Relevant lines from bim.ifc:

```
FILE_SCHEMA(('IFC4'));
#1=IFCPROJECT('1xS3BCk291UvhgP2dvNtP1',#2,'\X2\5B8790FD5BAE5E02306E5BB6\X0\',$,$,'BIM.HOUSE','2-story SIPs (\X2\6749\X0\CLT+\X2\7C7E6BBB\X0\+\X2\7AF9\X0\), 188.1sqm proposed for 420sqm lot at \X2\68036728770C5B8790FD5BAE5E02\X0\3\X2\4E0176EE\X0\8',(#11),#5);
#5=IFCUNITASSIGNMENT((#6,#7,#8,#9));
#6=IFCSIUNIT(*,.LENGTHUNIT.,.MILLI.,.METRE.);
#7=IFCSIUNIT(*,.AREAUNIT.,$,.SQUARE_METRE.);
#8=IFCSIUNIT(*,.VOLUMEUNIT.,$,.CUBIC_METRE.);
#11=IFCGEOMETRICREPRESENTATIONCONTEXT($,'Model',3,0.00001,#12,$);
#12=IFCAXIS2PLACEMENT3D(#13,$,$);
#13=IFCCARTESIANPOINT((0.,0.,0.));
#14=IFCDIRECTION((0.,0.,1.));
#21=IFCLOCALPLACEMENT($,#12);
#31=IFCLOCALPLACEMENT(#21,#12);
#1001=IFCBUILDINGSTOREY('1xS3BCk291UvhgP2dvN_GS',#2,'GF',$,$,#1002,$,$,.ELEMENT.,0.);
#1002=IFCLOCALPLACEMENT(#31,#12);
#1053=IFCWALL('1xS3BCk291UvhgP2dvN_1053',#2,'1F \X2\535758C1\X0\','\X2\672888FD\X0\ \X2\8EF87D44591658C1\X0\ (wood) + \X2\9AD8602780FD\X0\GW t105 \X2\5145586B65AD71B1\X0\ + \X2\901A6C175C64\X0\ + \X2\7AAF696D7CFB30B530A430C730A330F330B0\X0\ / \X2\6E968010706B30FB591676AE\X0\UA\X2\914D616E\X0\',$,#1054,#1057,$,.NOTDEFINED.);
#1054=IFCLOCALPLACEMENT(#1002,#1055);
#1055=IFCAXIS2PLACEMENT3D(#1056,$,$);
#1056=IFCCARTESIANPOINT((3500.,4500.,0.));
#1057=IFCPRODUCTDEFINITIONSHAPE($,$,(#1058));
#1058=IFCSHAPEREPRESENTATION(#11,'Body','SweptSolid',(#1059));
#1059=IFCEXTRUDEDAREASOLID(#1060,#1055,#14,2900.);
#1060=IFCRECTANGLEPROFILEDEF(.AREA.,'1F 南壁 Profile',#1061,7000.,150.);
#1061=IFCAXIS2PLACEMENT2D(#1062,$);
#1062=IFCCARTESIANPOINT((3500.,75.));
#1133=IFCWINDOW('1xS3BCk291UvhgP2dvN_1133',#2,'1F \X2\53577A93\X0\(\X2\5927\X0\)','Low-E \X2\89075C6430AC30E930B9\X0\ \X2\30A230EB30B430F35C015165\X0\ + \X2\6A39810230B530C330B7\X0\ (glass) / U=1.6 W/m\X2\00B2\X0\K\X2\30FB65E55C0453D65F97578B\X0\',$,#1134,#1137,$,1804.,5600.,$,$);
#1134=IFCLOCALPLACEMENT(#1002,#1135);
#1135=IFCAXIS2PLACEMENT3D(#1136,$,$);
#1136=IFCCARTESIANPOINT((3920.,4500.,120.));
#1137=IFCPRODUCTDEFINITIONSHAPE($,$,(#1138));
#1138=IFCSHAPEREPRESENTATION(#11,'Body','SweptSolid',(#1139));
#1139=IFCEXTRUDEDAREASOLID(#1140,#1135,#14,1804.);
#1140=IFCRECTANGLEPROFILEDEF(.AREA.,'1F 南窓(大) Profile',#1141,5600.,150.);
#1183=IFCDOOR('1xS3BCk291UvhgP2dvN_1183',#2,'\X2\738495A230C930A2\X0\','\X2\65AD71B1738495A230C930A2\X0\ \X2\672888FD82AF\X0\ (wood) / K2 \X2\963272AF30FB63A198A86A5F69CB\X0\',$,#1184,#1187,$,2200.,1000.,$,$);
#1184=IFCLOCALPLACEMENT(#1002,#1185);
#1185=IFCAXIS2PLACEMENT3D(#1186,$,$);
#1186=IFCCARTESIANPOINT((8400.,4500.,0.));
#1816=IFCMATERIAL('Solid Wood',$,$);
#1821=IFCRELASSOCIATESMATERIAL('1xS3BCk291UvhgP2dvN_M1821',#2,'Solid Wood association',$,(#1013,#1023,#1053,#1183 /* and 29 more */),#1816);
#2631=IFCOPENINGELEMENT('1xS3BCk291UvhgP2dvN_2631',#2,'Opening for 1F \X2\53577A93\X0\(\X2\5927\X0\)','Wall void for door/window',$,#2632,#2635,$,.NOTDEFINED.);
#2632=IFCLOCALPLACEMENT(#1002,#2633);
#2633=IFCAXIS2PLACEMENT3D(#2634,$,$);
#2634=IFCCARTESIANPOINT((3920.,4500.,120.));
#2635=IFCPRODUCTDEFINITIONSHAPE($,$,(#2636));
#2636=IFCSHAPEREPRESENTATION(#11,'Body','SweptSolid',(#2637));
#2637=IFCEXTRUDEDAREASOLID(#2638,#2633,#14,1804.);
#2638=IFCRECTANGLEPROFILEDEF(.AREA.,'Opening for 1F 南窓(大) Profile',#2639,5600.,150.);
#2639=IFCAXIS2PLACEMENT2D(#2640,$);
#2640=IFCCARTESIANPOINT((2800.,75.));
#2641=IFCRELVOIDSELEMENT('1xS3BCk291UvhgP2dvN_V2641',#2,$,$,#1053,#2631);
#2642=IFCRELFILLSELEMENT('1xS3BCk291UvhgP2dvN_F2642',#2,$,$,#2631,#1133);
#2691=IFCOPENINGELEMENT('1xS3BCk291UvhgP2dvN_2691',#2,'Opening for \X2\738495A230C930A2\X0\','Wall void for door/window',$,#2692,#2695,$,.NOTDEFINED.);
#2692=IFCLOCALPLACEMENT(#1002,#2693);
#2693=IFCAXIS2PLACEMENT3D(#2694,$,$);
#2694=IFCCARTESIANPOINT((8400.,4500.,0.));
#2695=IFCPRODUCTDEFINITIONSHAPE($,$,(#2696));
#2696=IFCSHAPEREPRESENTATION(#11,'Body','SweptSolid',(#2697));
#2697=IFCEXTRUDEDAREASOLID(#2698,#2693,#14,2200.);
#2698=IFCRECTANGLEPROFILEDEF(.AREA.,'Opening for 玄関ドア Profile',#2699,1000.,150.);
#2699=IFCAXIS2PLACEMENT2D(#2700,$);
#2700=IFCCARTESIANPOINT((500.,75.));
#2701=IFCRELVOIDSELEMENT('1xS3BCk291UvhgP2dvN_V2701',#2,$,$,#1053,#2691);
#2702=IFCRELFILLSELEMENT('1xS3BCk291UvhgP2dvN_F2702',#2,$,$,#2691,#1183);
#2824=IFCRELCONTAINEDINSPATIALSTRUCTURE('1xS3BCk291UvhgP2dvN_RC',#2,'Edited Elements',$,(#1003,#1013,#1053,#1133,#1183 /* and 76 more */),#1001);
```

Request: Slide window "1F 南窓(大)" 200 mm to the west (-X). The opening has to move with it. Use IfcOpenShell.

```python
import ifcopenshell
import ifcopenshell.api.geometry
import ifcopenshell.util.placement
import ifcopenshell.util.unit

model = ifcopenshell.open("bim.ifc")
unit_scale = ifcopenshell.util.unit.calculate_unit_scale(model)

window = model.by_guid("1xS3BCk291UvhgP2dvN_1133")
opening = window.FillsVoids[0].RelatingOpeningElement
wall = opening.VoidsElements[0].RelatingBuildingElement

wall_matrix = ifcopenshell.util.placement.get_local_placement(wall.ObjectPlacement)
shift = wall_matrix[:3, 0] * -0.2 / unit_scale
before = ifcopenshell.util.placement.get_local_placement(window.ObjectPlacement)[:3, 3].copy()

# The window is not placed relative to its opening, so move both.
for product in (opening, window):
    matrix = ifcopenshell.util.placement.get_local_placement(product.ObjectPlacement)
    matrix[:3, 3] += shift
    ifcopenshell.api.geometry.edit_object_placement(model, product=product, matrix=matrix, is_si=False)

after = ifcopenshell.util.placement.get_local_placement(window.ObjectPlacement)[:3, 3]
print("window moved by", (after - before).round(3) + 0.0)

model.write("bim-out.ifc")
```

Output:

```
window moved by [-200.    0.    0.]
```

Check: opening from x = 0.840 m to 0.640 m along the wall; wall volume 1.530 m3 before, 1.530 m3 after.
